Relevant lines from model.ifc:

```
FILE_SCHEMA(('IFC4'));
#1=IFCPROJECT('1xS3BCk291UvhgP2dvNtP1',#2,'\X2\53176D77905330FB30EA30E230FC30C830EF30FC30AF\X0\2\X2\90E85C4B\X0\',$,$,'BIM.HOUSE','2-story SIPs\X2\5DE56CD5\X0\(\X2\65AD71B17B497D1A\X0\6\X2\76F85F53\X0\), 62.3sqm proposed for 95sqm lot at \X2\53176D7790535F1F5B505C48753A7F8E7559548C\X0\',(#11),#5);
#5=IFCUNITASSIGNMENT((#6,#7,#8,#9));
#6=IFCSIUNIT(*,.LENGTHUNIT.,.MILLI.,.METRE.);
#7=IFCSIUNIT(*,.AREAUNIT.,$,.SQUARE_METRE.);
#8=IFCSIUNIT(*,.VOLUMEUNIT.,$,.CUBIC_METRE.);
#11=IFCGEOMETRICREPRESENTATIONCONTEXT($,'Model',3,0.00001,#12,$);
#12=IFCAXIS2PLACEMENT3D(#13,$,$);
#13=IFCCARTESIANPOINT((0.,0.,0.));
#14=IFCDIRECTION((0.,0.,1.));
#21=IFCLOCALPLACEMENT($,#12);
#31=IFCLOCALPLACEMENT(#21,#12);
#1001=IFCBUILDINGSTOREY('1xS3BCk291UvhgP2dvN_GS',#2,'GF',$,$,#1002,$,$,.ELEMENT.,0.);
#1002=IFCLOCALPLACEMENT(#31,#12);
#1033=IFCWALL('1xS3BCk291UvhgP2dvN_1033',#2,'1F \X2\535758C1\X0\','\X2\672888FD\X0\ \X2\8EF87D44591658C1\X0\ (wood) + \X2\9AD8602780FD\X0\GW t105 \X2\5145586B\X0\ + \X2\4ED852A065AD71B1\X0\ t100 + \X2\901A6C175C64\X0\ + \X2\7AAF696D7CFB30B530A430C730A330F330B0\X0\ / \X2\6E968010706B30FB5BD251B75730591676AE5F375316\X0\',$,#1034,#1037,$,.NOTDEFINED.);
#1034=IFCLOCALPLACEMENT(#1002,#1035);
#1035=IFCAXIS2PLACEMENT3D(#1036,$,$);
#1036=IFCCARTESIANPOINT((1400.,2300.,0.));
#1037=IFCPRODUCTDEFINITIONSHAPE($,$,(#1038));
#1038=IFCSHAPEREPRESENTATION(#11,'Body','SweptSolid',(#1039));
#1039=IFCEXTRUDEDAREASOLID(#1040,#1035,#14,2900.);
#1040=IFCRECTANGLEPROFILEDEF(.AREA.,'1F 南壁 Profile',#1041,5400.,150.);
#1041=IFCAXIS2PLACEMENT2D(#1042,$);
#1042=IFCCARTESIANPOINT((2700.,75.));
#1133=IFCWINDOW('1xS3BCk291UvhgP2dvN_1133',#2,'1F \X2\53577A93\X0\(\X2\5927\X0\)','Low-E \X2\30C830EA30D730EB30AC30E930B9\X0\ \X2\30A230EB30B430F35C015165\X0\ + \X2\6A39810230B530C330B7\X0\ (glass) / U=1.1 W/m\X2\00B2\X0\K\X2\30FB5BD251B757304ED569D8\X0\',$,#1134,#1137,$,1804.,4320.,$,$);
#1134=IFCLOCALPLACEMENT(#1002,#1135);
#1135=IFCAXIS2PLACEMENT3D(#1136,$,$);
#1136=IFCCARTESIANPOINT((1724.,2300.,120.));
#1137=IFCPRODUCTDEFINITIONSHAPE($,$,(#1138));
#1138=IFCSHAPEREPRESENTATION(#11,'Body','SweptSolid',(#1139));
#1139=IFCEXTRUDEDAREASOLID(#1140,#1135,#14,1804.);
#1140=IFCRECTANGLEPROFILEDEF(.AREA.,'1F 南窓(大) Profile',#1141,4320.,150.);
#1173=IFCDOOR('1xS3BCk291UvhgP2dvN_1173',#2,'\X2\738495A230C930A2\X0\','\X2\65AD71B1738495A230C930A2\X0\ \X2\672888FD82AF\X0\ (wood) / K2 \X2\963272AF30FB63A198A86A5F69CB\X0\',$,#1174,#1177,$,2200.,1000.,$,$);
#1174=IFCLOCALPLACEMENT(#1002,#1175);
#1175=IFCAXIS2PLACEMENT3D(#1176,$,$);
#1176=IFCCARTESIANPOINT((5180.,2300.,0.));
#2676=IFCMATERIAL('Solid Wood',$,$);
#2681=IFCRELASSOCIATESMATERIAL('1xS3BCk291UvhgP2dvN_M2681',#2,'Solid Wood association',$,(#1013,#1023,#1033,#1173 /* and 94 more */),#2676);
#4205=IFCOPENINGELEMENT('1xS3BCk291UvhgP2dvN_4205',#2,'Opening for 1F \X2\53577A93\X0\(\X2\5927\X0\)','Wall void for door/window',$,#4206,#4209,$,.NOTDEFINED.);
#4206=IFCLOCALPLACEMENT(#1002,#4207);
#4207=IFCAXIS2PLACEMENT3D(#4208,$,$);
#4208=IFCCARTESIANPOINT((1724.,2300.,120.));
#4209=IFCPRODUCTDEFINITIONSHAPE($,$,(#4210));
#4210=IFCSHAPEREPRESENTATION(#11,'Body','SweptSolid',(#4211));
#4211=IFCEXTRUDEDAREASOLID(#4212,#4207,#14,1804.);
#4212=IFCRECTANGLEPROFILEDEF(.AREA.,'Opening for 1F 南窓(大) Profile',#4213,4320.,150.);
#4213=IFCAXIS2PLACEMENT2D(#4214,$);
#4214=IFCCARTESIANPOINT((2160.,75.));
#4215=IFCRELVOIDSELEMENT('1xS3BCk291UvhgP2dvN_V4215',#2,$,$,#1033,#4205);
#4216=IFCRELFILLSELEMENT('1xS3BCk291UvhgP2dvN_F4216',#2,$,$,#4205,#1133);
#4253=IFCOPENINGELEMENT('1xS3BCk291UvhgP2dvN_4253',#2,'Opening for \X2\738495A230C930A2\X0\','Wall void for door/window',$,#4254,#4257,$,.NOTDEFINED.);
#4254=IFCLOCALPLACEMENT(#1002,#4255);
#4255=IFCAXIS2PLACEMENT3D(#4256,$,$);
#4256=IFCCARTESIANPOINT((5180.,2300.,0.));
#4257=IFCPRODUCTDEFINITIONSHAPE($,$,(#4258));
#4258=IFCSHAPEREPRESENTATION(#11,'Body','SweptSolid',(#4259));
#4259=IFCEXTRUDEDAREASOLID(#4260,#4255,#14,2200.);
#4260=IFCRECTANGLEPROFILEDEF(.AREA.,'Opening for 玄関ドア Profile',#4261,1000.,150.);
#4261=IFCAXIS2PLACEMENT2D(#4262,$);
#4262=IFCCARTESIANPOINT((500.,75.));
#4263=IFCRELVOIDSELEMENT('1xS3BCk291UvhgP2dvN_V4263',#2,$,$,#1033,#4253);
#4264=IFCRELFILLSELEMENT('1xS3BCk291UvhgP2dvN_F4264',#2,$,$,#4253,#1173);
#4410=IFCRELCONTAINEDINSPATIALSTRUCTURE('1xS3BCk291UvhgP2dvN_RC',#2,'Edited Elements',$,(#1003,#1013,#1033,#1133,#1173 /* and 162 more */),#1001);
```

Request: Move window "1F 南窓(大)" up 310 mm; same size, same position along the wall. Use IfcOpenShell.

```python
import numpy as np
import ifcopenshell
import ifcopenshell.api.geometry
import ifcopenshell.util.placement
import ifcopenshell.util.unit

model = ifcopenshell.open("model.ifc")
unit_scale = ifcopenshell.util.unit.calculate_unit_scale(model)

window = model.by_guid("1xS3BCk291UvhgP2dvN_1133")
opening = window.FillsVoids[0].RelatingOpeningElement
dz = 310.0

shift = np.array([0.0, 0.0, dz])
# The window is not placed relative to its opening, so move both.
for product in (opening, window):
    matrix = ifcopenshell.util.placement.get_local_placement(product.ObjectPlacement)
    matrix[:3, 3] += shift
    ifcopenshell.api.geometry.edit_object_placement(model, product=product, matrix=matrix, is_si=False)

print(f"moved by {dz * unit_scale:+.3f} m")

model.write("model_edited.ifc")
```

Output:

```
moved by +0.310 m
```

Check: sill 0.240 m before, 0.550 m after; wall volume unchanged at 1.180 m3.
